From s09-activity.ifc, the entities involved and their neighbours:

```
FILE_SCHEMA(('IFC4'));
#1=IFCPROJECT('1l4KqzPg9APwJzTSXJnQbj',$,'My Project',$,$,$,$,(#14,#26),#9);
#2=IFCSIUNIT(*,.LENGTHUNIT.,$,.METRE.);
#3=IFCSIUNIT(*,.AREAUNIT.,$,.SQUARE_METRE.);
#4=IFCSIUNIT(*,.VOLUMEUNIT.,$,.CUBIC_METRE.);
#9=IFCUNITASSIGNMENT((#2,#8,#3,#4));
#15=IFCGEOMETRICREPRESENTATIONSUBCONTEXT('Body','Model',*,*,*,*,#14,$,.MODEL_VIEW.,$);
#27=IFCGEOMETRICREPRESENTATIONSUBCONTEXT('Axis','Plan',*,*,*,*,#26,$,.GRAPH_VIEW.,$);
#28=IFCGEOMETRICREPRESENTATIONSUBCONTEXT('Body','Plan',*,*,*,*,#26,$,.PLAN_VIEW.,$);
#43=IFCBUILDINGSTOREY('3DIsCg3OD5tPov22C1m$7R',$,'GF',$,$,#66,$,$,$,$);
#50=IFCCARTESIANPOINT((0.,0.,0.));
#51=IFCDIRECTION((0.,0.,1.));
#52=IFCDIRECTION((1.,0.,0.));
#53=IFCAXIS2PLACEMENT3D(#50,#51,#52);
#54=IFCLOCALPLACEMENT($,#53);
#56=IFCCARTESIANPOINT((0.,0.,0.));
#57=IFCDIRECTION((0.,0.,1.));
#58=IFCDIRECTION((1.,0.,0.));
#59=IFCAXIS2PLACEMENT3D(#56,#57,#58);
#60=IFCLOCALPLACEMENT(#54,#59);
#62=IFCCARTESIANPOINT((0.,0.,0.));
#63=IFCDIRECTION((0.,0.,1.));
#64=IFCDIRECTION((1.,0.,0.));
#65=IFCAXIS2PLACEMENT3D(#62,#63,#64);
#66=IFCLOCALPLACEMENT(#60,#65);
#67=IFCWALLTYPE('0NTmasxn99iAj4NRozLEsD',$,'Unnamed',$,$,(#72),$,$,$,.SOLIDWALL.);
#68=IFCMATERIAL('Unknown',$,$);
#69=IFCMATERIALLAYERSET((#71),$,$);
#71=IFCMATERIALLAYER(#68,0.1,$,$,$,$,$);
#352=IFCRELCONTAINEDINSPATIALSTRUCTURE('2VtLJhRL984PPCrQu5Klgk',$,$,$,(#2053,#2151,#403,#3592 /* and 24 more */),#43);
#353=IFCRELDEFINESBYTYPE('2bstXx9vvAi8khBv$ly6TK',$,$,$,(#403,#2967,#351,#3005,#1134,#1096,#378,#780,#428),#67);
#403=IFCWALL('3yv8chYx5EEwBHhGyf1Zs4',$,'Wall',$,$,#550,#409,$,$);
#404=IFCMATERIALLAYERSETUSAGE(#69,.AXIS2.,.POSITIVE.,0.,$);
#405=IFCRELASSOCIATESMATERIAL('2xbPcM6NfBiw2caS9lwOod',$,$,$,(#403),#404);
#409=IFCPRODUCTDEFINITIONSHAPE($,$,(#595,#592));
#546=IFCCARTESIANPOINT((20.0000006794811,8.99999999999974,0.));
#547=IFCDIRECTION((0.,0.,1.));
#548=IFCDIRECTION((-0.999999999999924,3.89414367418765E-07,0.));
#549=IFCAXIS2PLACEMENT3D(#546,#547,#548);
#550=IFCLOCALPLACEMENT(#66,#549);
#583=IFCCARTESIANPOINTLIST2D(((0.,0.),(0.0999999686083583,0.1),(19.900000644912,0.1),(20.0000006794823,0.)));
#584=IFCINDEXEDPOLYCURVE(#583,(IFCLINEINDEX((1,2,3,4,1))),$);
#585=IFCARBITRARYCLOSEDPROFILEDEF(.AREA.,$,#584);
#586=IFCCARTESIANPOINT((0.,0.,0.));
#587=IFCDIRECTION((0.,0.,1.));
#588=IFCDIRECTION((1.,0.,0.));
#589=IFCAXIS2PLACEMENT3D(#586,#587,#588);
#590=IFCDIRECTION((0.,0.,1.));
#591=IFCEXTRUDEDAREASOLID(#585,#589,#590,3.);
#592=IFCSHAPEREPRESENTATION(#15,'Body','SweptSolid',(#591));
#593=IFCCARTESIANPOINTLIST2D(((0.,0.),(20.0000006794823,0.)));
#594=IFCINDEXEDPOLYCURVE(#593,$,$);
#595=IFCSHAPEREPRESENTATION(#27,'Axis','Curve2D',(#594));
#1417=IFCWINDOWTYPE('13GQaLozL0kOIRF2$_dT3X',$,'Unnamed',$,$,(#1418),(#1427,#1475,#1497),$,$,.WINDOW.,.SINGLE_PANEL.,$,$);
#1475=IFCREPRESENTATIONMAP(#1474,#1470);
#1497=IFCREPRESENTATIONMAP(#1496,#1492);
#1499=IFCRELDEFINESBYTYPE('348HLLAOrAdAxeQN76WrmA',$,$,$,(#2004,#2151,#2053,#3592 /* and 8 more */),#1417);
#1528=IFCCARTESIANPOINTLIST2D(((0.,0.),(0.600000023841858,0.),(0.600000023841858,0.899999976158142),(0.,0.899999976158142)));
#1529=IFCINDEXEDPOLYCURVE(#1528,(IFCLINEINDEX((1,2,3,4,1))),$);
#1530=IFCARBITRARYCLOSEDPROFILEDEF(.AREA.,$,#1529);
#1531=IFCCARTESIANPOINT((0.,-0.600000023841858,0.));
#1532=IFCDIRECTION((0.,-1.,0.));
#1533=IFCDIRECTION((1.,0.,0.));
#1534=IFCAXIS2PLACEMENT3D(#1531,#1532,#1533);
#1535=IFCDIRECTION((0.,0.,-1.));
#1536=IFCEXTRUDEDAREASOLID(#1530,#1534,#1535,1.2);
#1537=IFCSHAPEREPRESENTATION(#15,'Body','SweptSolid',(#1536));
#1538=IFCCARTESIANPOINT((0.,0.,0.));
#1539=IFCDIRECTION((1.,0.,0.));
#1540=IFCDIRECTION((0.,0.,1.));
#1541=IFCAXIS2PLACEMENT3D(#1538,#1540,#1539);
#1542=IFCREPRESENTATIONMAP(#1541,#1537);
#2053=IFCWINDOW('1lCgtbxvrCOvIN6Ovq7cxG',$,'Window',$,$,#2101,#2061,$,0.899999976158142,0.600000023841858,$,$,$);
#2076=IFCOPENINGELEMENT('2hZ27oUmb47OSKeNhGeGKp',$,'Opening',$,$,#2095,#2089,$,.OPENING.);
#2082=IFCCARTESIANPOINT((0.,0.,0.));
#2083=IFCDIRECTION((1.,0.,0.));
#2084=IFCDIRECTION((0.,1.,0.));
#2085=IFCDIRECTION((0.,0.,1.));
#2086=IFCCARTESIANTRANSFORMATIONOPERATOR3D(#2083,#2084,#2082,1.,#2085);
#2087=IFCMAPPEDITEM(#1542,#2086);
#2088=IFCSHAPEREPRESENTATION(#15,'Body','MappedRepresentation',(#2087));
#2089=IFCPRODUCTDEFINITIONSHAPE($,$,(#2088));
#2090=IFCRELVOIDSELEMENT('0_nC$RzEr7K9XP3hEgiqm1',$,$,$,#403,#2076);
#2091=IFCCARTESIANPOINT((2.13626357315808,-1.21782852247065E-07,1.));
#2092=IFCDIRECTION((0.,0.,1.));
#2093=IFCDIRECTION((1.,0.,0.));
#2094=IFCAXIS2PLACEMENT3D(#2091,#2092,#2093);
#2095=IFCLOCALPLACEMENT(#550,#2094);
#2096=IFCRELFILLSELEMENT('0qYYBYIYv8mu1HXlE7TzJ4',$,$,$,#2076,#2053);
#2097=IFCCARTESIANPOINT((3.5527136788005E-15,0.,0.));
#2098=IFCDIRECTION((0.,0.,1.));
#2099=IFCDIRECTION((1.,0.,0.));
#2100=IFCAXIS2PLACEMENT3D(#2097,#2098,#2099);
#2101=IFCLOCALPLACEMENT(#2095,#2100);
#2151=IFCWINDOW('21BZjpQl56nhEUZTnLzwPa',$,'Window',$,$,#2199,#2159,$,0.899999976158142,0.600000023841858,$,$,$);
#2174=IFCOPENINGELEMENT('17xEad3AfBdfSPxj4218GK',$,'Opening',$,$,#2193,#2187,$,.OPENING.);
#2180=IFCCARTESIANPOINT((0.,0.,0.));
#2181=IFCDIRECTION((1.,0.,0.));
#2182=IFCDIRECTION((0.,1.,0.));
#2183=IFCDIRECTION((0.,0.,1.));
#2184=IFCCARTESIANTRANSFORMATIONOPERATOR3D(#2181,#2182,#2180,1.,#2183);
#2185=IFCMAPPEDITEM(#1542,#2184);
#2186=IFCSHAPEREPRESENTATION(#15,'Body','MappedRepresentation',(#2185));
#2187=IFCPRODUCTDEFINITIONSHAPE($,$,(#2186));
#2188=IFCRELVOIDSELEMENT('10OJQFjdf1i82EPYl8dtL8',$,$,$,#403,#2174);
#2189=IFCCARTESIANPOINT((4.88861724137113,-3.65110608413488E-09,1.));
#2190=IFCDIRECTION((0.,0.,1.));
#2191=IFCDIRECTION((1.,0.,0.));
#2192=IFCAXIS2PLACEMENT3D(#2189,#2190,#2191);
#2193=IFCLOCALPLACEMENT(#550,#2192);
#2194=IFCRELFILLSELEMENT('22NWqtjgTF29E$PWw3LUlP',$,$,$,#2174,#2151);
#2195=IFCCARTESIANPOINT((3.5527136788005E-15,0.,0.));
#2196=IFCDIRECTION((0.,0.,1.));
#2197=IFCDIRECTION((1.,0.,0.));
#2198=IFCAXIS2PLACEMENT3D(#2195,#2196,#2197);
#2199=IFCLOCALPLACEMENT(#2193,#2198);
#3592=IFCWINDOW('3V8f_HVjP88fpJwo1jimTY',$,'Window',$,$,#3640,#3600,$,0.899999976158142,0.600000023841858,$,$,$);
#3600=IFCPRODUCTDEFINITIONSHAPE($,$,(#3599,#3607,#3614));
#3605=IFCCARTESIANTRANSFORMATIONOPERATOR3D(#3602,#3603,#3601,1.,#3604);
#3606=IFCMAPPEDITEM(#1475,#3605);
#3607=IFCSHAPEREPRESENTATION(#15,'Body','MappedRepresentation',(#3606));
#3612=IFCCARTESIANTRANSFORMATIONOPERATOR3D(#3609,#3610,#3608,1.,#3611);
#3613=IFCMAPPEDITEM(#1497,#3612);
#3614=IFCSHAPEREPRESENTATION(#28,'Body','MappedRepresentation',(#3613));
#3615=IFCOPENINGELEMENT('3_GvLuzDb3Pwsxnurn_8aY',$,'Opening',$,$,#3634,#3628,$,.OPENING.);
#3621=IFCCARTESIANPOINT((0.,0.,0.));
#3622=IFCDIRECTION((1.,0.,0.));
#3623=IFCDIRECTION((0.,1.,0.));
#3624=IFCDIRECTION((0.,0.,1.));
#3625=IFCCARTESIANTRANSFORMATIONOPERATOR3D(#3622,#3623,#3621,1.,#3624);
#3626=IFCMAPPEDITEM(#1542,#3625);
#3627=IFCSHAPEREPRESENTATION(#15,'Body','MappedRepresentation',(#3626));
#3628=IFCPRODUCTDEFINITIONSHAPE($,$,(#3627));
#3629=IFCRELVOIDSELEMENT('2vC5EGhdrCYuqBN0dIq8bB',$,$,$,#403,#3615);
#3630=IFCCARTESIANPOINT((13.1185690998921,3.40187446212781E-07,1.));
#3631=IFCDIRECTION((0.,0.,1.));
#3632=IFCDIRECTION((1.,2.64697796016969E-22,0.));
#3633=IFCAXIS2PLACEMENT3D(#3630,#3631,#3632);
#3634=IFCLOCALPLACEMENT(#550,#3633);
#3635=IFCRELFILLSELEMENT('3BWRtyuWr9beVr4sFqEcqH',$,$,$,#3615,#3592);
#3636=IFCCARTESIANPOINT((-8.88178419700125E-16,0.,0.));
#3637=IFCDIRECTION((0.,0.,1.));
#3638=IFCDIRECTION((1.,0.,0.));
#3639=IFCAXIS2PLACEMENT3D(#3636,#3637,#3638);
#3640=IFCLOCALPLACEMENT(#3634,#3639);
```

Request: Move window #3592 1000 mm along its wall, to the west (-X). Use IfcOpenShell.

```python
import ifcopenshell
import ifcopenshell.api.geometry
import ifcopenshell.util.placement
import ifcopenshell.util.unit

model = ifcopenshell.open("s09-activity.ifc")
unit_scale = ifcopenshell.util.unit.calculate_unit_scale(model)

window = model.by_guid("3V8f_HVjP88fpJwo1jimTY")
opening = window.FillsVoids[0].RelatingOpeningElement
wall = opening.VoidsElements[0].RelatingBuildingElement

wall_matrix = ifcopenshell.util.placement.get_local_placement(wall.ObjectPlacement)
shift = wall_matrix[:3, 0] * 1 / unit_scale
before = ifcopenshell.util.placement.get_local_placement(window.ObjectPlacement)[:3, 3].copy()

# The window is placed relative to its opening, so it follows when the opening moves.
matrix = ifcopenshell.util.placement.get_local_placement(opening.ObjectPlacement)
matrix[:3, 3] += shift
ifcopenshell.api.geometry.edit_object_placement(
    model, product=opening, matrix=matrix, is_si=False, should_transform_children=True
)

after = ifcopenshell.util.placement.get_local_placement(window.ObjectPlacement)[:3, 3]
print("window moved by", (after - before).round(3) + 0.0)

model.write("s09-activity_updated.ifc")
```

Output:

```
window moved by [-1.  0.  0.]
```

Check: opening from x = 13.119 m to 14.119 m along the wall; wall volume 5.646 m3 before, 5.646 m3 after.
